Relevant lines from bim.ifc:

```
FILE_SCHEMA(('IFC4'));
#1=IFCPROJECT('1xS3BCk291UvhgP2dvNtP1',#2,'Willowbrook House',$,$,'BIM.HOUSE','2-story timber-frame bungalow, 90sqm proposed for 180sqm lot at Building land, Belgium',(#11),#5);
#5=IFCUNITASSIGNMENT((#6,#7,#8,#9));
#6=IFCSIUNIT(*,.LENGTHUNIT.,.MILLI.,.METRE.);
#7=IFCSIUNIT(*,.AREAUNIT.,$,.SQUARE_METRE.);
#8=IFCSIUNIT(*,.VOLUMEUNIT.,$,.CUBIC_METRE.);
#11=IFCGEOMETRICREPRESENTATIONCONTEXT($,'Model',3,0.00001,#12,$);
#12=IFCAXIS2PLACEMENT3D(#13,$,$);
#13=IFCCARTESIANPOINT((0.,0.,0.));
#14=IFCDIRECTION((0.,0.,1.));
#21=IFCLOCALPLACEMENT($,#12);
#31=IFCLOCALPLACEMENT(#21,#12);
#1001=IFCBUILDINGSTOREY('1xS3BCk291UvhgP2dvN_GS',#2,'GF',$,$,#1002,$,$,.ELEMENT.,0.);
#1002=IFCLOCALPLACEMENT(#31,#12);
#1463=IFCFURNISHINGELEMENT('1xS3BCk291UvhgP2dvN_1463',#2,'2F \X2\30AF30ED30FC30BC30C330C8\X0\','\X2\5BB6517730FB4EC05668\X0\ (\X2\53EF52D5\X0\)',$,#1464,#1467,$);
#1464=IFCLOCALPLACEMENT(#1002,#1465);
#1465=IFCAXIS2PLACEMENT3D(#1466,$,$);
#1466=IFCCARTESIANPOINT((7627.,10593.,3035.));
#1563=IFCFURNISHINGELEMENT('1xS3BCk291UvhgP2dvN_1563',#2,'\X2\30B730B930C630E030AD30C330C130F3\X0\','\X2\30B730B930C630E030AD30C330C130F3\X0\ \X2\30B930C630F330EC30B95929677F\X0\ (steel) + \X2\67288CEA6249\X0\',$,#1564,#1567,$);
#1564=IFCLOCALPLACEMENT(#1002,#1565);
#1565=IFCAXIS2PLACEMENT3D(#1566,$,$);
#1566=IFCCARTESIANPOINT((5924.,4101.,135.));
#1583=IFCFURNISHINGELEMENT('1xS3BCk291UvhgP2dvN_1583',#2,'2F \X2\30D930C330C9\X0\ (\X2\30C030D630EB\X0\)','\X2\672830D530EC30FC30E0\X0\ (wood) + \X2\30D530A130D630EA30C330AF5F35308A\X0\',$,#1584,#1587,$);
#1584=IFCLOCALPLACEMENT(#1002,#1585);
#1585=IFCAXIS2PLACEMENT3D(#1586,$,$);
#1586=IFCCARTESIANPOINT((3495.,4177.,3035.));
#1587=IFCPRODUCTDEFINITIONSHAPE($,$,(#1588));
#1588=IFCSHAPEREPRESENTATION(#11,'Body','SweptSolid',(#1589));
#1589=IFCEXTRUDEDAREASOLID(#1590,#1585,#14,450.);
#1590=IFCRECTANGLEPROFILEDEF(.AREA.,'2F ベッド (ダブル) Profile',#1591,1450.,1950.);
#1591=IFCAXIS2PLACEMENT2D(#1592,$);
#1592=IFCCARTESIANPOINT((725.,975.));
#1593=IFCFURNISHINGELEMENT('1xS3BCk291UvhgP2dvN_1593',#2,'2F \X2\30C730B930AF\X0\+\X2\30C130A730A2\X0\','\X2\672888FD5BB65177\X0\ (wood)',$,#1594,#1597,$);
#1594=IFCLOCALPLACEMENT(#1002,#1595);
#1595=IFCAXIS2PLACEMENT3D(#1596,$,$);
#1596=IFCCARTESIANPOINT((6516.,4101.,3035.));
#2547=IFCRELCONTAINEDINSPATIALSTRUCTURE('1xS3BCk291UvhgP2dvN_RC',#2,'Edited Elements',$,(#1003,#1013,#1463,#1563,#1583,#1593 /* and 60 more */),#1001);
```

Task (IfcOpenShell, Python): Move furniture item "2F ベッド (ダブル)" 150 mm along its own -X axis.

```python
import ifcopenshell
import ifcopenshell.api.geometry
import ifcopenshell.util.placement
import ifcopenshell.util.unit

model = ifcopenshell.open("bim.ifc")
unit_scale = ifcopenshell.util.unit.calculate_unit_scale(model)

item = model.by_guid("1xS3BCk291UvhgP2dvN_1583")
matrix = ifcopenshell.util.placement.get_local_placement(item.ObjectPlacement)
matrix[:3, 3] -= matrix[:3, 0] * 0.15 / unit_scale
ifcopenshell.api.geometry.edit_object_placement(model, product=item, matrix=matrix, is_si=False)

print(ifcopenshell.util.placement.get_local_placement(item.ObjectPlacement).round(3) + 0.0)

model.write("bim_updated.ifc")
```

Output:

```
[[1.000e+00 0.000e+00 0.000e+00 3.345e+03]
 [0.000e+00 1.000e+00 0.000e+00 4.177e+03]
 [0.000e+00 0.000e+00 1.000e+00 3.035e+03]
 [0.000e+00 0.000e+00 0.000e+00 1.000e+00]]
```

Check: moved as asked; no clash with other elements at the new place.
